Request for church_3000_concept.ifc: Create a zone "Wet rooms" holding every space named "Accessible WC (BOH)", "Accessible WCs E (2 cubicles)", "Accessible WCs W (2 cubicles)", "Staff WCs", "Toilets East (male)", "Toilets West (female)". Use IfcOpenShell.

First a look at what the model holds.

```python
import ifcopenshell

model = ifcopenshell.open("church_3000_concept.ifc")
print(model.schema)
seen = {}
for space in model.by_type("IfcSpace"):
    seen[space.LongName] = seen.get(space.LongName, 0) + 1
for name, count in sorted(seen.items(), key=str):
    print(count, "x", name)
print("zones:", [z.Name for z in model.by_type("IfcZone")][:20])
```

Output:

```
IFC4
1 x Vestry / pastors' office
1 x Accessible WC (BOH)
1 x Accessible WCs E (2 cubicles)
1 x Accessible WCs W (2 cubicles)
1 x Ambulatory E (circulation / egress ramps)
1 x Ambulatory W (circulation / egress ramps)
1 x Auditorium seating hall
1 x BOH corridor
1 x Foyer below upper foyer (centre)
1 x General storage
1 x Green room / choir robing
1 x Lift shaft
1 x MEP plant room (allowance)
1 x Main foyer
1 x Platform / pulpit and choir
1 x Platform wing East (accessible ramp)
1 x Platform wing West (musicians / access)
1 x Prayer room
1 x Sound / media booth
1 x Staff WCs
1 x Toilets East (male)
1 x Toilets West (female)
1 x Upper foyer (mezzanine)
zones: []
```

```python
import ifcopenshell
import ifcopenshell.api.group
import ifcopenshell.api.root

model = ifcopenshell.open("church_3000_concept.ifc")

names = {"Accessible WC (BOH)", "Accessible WCs E (2 cubicles)", "Accessible WCs W (2 cubicles)", "Staff WCs", "Toilets East (male)", "Toilets West (female)"}
spaces = [s for s in model.by_type("IfcSpace") if s.LongName in names]

zone = ifcopenshell.api.root.create_entity(model, ifc_class="IfcZone", name="Wet rooms")
ifcopenshell.api.group.assign_group(model, products=spaces, group=zone)
print(len(spaces), "spaces in", zone.Name)

model.write("church_3000_concept_updated.ifc")
```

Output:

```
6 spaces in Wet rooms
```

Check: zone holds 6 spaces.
